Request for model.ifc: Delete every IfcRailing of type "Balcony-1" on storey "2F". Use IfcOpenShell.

First a look at what the model holds.

```python
import ifcopenshell
import ifcopenshell.util.element

model = ifcopenshell.open("model.ifc")
print(model.schema)
storey = next(s for s in model.by_type("IfcBuildingStorey") if s.Name == "2F")
railings = [e for e in ifcopenshell.util.element.get_decomposition(storey) if e.is_a("IfcRailing")]
seen = {}
for e in railings:
    element_type = ifcopenshell.util.element.get_type(e)
    name = element_type.Name if element_type not in (None, e) else None
    seen[name] = seen.get(name, 0) + 1
for name, count in sorted(seen.items(), key=str):
    print(count, "x", name)
```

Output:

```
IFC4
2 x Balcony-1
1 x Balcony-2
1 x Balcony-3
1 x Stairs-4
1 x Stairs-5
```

```python
import ifcopenshell
import ifcopenshell.api.root
import ifcopenshell.util.element

model = ifcopenshell.open("model.ifc")

storey = next(s for s in model.by_type("IfcBuildingStorey") if s.Name == "2F")
railings = [e for e in ifcopenshell.util.element.get_decomposition(storey) if e.is_a("IfcRailing")]
targets = [e for e in railings if (t := ifcopenshell.util.element.get_type(e)) not in (None, e) and t.Name == "Balcony-1"]

for e in targets:
    ifcopenshell.api.root.remove_product(model, product=e)
print(len(targets), "removed")

model.write("model_rev.ifc")
```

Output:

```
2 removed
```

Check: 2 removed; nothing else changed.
